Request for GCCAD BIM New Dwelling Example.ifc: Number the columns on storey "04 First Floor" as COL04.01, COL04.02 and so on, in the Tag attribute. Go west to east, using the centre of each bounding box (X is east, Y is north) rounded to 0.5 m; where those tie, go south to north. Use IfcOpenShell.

First a look at what the model holds.

```python
import ifcopenshell
import ifcopenshell.util.element
import ifcopenshell.util.placement

model = ifcopenshell.open("GCCAD BIM New Dwelling Example.ifc")
print(model.schema)
storey = next(s for s in model.by_type("IfcBuildingStorey") if s.Name == "04 First Floor")
columns = [e for e in ifcopenshell.util.element.get_decomposition(storey) if e.is_a("IfcColumn")]
for e in sorted(columns, key=lambda e: e.id()):
    origin = ifcopenshell.util.placement.get_local_placement(e.ObjectPlacement)[:3, 3]
    print(e.id(), e.Tag, e.Name, origin.round(2) + 0.0, sep=" | ")
```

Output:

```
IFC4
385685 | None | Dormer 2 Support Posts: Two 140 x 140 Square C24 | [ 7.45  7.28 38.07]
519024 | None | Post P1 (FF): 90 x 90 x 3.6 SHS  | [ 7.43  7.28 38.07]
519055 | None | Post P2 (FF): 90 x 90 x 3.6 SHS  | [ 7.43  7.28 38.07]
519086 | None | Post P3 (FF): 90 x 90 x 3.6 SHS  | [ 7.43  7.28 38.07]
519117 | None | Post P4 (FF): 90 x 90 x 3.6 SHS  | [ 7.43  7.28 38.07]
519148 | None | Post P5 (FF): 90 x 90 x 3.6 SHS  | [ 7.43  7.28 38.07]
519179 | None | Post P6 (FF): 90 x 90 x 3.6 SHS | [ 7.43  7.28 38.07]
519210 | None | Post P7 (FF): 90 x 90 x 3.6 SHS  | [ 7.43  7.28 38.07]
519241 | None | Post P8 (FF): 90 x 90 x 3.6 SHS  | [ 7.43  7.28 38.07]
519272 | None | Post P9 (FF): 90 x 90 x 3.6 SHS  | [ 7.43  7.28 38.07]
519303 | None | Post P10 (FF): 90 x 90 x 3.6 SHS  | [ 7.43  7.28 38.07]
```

```python
import ifcopenshell
import ifcopenshell.geom
import ifcopenshell.util.element
import ifcopenshell.util.shape

model = ifcopenshell.open("GCCAD BIM New Dwelling Example.ifc")
settings = ifcopenshell.geom.settings()
settings.set("use-world-coords", True)


def centre(element):
    shape = ifcopenshell.geom.create_shape(settings, element)
    return ifcopenshell.util.shape.get_bbox_centroid(shape.geometry)


storey = next(s for s in model.by_type("IfcBuildingStorey") if s.Name == "04 First Floor")
columns = [e for e in ifcopenshell.util.element.get_decomposition(storey) if e.is_a("IfcColumn")]

# Insertion points can sit at a corner or the storey origin, so sort by the geometry (in metres).
centres = {e: centre(e) for e in columns}
columns.sort(key=lambda e: (round(centres[e][0] / 0.5), centres[e][1]))

for i, e in enumerate(columns, start=1):
    number = f"COL04.{i:02d}"
    e.Tag = number
    print(e.id(), number)

model.write("GCCAD BIM New Dwelling Example-out.ifc")
```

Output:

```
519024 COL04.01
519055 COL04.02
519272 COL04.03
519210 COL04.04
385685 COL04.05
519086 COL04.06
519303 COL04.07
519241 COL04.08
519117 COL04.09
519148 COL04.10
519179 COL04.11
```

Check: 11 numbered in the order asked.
